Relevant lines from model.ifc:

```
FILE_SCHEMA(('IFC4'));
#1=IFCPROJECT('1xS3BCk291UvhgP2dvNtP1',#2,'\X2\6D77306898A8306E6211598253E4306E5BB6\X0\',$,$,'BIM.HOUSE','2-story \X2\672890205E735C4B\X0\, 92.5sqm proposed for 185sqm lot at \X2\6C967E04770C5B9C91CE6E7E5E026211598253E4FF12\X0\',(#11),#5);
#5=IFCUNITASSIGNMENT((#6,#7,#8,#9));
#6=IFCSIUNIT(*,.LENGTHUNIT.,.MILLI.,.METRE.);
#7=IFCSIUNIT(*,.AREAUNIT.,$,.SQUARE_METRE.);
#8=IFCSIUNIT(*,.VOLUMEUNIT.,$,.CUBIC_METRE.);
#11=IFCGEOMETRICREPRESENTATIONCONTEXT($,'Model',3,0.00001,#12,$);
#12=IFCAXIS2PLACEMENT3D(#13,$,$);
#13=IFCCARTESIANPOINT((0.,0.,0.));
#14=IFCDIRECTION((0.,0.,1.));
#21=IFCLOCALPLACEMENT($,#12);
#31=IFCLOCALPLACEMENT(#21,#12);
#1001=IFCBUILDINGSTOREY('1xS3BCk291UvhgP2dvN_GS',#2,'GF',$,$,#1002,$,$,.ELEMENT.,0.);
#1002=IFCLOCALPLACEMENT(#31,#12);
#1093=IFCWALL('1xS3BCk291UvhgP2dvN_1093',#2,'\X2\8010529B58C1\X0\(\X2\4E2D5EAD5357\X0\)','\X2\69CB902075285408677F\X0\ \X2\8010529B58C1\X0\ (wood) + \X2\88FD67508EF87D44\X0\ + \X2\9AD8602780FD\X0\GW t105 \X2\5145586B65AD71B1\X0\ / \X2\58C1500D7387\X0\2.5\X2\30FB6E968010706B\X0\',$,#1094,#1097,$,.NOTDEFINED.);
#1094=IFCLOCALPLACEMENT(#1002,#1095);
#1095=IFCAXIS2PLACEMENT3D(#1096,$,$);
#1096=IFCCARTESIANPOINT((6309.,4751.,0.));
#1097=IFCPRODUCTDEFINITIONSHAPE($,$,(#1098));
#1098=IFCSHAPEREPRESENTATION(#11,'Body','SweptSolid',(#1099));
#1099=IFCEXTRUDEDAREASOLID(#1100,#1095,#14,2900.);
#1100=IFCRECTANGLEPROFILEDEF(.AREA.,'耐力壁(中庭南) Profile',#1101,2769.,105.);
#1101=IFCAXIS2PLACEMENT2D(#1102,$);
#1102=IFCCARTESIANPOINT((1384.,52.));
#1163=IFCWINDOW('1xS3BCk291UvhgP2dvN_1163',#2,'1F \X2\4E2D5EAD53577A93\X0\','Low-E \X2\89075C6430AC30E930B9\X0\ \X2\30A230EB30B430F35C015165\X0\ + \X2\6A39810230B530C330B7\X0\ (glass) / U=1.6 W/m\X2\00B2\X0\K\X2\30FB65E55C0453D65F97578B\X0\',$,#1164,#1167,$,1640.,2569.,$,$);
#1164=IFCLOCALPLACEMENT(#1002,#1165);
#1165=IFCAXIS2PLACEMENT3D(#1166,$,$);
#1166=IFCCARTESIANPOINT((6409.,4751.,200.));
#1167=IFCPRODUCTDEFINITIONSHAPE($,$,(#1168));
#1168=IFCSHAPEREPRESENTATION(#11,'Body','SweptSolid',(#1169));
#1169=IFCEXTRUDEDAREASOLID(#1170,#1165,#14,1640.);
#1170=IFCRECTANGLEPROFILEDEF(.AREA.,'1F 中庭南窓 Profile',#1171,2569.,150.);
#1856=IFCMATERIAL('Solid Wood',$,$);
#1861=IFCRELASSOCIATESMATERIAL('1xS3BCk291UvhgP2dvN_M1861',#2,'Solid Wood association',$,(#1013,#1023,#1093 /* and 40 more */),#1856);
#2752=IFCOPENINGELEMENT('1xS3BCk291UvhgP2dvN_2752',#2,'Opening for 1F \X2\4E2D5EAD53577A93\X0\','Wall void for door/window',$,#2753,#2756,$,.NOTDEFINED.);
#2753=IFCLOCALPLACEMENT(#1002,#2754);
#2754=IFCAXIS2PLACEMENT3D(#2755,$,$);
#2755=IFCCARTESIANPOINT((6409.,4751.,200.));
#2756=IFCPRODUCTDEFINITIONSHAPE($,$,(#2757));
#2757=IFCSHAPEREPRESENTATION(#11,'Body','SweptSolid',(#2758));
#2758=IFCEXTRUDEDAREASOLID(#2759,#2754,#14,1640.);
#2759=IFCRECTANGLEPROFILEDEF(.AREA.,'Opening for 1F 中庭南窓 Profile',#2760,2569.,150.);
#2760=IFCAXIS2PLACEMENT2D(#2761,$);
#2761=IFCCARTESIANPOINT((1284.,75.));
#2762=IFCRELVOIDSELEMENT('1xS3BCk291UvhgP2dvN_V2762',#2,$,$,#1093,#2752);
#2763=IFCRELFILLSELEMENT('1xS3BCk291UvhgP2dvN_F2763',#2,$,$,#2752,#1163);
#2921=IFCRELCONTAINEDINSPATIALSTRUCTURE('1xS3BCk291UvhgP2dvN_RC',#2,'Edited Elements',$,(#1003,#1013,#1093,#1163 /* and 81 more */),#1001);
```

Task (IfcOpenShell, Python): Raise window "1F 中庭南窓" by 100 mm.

```python
import numpy as np
import ifcopenshell
import ifcopenshell.api.geometry
import ifcopenshell.util.placement
import ifcopenshell.util.unit

model = ifcopenshell.open("model.ifc")
unit_scale = ifcopenshell.util.unit.calculate_unit_scale(model)

window = model.by_id(1163)
opening = window.FillsVoids[0].RelatingOpeningElement
dz = 100.0

shift = np.array([0.0, 0.0, dz])
# The window is not placed relative to its opening, so move both.
for product in (opening, window):
    matrix = ifcopenshell.util.placement.get_local_placement(product.ObjectPlacement)
    matrix[:3, 3] += shift
    ifcopenshell.api.geometry.edit_object_placement(model, product=product, matrix=matrix, is_si=False)

print(f"moved by {dz * unit_scale:+.3f} m")

model.write("model_edited.ifc")
```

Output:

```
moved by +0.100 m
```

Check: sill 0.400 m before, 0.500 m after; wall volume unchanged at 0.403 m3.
